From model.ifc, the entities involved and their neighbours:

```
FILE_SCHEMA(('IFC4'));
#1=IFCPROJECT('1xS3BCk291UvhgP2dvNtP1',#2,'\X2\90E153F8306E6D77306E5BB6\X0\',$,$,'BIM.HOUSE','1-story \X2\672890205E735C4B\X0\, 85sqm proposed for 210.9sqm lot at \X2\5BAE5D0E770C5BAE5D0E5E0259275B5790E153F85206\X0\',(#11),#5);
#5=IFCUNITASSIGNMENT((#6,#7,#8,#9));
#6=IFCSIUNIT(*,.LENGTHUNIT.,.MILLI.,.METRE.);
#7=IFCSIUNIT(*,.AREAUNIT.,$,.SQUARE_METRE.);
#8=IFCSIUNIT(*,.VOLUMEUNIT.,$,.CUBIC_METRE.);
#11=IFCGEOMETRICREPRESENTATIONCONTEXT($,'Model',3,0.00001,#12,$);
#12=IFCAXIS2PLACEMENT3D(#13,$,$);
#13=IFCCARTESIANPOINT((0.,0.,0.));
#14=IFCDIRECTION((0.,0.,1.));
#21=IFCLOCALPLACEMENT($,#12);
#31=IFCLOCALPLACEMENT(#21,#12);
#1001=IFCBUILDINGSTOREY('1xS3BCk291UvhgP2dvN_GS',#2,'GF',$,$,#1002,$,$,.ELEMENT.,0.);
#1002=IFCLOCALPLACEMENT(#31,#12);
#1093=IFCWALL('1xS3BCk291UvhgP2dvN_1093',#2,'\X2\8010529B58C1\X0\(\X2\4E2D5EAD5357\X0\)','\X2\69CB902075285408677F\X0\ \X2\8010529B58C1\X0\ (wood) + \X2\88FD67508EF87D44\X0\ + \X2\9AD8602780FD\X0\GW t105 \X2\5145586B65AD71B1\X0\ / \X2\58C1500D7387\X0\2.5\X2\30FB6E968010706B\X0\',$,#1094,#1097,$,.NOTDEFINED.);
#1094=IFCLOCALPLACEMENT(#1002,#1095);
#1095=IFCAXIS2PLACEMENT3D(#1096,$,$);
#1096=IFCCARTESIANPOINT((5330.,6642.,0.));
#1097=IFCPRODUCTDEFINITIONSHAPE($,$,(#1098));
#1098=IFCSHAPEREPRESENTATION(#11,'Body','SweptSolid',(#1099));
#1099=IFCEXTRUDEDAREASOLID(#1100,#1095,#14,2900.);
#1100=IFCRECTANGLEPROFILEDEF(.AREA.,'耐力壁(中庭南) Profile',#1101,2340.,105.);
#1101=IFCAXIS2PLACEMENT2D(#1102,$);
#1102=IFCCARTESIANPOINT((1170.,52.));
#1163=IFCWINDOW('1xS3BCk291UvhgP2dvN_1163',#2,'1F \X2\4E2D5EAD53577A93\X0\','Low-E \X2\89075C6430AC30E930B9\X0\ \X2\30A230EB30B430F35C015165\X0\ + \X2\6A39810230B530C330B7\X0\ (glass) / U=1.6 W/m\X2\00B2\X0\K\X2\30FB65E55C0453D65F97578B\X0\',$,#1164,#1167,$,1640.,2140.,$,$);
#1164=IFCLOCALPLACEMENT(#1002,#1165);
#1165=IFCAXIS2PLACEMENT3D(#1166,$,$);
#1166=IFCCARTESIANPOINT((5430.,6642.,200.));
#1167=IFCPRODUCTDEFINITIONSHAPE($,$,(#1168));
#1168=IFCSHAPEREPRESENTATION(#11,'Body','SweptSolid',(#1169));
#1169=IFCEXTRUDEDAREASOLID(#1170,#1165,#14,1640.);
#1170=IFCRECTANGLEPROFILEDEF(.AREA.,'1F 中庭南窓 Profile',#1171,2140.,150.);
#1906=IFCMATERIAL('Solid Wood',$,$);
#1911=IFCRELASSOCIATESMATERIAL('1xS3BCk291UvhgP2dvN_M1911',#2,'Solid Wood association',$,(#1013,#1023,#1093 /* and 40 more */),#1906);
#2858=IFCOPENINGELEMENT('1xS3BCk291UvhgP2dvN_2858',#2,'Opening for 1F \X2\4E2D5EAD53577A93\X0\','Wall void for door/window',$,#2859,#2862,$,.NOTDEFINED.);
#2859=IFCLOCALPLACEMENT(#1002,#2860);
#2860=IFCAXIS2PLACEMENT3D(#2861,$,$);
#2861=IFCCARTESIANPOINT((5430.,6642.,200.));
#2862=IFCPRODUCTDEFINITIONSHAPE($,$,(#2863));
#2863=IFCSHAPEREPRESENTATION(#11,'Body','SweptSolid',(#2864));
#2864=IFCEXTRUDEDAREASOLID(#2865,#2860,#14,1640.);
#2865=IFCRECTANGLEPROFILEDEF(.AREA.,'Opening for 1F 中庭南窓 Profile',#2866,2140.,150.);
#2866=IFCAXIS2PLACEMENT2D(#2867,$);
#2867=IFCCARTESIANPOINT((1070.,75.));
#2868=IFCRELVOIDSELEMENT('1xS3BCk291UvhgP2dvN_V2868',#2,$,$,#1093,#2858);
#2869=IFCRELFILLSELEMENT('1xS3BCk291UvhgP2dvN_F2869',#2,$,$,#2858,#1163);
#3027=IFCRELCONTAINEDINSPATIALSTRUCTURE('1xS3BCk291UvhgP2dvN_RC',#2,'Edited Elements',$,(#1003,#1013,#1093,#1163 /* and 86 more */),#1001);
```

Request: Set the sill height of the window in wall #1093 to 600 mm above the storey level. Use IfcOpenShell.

```python
import numpy as np
import ifcopenshell
import ifcopenshell.api.geometry
import ifcopenshell.geom
import ifcopenshell.util.element
import ifcopenshell.util.placement
import ifcopenshell.util.shape
import ifcopenshell.util.unit

model = ifcopenshell.open("model.ifc")
unit_scale = ifcopenshell.util.unit.calculate_unit_scale(model)

window = model.by_guid("1xS3BCk291UvhgP2dvN_1163")
opening = window.FillsVoids[0].RelatingOpeningElement
storey = ifcopenshell.util.element.get_container(window, ifc_class="IfcBuildingStorey")
level = ifcopenshell.util.placement.get_local_placement(storey.ObjectPlacement)[2, 3]

# The opening's origin need not be at the sill, so measure its lowest point.
shape = ifcopenshell.geom.create_shape(ifcopenshell.geom.settings(), opening)
bottom = ifcopenshell.util.shape.get_shape_bottom_elevation(shape, shape.geometry) / unit_scale
dz = level + 600.0 - bottom

shift = np.array([0.0, 0.0, dz])
# The window is not placed relative to its opening, so move both.
for product in (opening, window):
    matrix = ifcopenshell.util.placement.get_local_placement(product.ObjectPlacement)
    matrix[:3, 3] += shift
    ifcopenshell.api.geometry.edit_object_placement(model, product=product, matrix=matrix, is_si=False)

print(f"moved by {dz * unit_scale:+.3f} m")

model.write("model_v2.ifc")
```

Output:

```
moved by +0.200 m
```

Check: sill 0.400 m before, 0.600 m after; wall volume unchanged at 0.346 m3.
